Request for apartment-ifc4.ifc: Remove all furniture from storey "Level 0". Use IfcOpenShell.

First a look at what the model holds.

```python
import ifcopenshell
import ifcopenshell.util.element

model = ifcopenshell.open("apartment-ifc4.ifc")
print(model.schema)
storey = next(s for s in model.by_type("IfcBuildingStorey") if s.Name == "Level 0")
furniture = [e for e in ifcopenshell.util.element.get_decomposition(storey) if e.is_a("IfcFurnishingElement")]
seen = {}
for e in furniture:
    element_type = ifcopenshell.util.element.get_type(e)
    name = element_type.Name if element_type not in (None, e) else None
    seen[name] = seen.get(name, 0) + 1
for name, count in sorted(seen.items(), key=str):
    print(count, "x", name)
```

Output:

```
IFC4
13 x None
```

```python
import ifcopenshell
import ifcopenshell.api.root
import ifcopenshell.util.element

model = ifcopenshell.open("apartment-ifc4.ifc")

storey = next(s for s in model.by_type("IfcBuildingStorey") if s.Name == "Level 0")
furniture = [e for e in ifcopenshell.util.element.get_decomposition(storey) if e.is_a("IfcFurnishingElement")]

for e in furniture:
    ifcopenshell.api.root.remove_product(model, product=e)
print(len(furniture), "removed")

model.write("apartment-ifc4_edited.ifc")
```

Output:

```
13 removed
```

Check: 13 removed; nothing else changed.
